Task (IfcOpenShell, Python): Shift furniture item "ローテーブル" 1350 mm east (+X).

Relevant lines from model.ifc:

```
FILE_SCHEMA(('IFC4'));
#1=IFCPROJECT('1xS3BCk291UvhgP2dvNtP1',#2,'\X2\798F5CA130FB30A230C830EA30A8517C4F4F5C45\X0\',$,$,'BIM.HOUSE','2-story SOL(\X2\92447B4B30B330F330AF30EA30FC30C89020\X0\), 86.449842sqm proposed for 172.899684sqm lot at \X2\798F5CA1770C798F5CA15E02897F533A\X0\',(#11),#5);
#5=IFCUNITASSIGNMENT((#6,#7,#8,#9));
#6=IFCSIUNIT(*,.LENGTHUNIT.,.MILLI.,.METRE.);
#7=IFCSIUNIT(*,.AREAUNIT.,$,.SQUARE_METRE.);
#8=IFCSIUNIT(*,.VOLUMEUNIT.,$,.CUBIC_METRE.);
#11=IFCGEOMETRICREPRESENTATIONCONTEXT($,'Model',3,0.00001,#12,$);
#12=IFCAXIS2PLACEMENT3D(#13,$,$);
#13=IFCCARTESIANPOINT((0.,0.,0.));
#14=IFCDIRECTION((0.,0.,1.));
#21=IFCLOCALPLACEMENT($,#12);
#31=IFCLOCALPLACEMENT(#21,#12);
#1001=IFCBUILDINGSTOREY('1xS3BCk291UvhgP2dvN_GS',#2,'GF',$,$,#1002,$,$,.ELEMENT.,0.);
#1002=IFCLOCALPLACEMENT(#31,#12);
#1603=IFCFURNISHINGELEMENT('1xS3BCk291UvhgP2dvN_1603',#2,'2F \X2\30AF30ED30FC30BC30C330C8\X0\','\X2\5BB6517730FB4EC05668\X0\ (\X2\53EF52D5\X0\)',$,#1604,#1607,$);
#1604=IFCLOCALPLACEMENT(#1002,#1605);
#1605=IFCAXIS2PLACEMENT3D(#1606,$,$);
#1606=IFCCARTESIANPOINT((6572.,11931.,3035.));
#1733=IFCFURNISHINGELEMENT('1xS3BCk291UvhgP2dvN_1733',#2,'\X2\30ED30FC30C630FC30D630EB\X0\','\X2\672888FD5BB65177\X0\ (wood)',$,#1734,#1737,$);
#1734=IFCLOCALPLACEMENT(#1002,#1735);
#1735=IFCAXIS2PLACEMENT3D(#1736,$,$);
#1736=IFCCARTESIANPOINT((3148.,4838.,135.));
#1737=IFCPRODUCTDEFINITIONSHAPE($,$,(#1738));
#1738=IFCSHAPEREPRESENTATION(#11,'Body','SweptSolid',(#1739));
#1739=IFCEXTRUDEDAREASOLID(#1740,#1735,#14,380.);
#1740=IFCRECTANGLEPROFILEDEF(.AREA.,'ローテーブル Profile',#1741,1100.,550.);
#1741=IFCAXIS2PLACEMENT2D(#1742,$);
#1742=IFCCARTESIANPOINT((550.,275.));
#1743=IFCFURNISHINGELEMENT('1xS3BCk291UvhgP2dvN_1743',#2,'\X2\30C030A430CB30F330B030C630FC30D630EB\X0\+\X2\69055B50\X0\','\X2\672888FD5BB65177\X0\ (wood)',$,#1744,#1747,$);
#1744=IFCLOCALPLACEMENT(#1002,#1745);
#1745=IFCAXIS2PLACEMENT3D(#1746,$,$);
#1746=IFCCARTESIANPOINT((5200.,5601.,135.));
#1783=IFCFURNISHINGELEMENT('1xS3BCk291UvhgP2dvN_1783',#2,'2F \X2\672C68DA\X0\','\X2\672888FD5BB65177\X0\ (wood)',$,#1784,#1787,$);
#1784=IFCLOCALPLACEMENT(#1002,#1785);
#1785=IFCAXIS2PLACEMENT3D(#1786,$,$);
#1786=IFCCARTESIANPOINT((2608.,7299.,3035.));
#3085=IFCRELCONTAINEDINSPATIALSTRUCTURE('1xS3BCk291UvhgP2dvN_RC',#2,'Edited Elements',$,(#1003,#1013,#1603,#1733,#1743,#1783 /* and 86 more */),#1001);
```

```python
import ifcopenshell
import ifcopenshell.api.geometry
import ifcopenshell.util.placement

model = ifcopenshell.open("model.ifc")

item = model.by_guid("1xS3BCk291UvhgP2dvN_1733")
matrix = ifcopenshell.util.placement.get_local_placement(item.ObjectPlacement)
matrix[0, 3] += 1350.0
ifcopenshell.api.geometry.edit_object_placement(model, product=item, matrix=matrix, is_si=False)

print(ifcopenshell.util.placement.get_local_placement(item.ObjectPlacement).round(3) + 0.0)

model.write("model-out.ifc")
```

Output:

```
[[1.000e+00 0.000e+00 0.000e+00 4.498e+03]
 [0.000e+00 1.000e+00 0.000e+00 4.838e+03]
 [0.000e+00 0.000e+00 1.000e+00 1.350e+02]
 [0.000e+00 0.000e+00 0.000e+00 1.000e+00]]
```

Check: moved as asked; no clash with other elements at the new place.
